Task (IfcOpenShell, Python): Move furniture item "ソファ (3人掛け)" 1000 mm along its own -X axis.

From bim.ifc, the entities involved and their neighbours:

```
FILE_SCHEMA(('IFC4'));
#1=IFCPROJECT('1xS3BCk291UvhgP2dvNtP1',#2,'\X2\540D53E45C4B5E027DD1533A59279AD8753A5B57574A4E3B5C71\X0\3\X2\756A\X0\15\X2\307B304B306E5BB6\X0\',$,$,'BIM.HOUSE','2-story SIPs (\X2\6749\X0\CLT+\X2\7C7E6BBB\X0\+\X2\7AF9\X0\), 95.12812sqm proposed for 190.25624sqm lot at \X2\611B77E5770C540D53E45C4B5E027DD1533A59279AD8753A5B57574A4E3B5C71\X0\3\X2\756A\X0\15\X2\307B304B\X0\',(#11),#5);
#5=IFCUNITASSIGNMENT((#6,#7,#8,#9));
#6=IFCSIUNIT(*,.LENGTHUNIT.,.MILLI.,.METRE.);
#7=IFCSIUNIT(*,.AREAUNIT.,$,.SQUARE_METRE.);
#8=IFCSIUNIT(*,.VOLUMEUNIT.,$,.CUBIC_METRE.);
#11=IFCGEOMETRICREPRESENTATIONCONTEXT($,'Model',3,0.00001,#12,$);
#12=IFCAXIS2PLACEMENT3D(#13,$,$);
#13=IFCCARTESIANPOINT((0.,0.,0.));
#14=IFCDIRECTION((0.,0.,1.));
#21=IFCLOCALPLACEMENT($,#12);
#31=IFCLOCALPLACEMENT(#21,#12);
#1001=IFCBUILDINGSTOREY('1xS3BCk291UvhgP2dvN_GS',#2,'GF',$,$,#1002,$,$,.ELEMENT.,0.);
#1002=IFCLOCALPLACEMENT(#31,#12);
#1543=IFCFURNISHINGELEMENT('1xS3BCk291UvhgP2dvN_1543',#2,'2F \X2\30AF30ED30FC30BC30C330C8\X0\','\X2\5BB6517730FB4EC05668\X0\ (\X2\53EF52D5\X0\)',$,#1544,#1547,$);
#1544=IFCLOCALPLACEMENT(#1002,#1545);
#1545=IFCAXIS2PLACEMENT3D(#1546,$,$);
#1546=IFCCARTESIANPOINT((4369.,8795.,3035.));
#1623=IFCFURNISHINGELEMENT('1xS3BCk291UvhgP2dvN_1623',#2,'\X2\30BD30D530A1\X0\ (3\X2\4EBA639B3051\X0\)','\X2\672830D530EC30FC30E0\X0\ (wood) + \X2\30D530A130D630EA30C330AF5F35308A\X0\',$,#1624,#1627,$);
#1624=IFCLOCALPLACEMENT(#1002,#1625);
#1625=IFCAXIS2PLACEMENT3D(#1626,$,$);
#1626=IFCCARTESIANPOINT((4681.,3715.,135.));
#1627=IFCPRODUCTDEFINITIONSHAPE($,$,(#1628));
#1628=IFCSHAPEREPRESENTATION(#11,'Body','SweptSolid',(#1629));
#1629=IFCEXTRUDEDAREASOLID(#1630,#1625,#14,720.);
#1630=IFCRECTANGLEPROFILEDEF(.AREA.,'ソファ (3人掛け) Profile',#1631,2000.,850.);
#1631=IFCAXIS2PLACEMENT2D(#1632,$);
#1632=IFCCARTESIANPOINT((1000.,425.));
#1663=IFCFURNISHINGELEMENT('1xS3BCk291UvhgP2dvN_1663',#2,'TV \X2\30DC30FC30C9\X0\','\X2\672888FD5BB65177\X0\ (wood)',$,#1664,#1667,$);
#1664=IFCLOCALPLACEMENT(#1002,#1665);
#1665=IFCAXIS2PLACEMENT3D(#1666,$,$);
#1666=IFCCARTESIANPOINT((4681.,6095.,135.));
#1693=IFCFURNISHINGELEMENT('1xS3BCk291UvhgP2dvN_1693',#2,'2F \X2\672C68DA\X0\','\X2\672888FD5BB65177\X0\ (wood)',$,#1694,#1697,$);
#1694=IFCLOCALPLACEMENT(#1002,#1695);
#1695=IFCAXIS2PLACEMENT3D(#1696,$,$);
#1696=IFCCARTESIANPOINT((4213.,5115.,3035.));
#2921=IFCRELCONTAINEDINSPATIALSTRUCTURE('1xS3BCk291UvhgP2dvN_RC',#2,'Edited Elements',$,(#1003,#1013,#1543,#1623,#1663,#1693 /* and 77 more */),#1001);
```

```python
import ifcopenshell
import ifcopenshell.api.geometry
import ifcopenshell.util.placement

model = ifcopenshell.open("bim.ifc")

item = model.by_id(1623)
matrix = ifcopenshell.util.placement.get_local_placement(item.ObjectPlacement)
matrix[:3, 3] -= matrix[:3, 0] * 1000.0
ifcopenshell.api.geometry.edit_object_placement(model, product=item, matrix=matrix, is_si=False)

print(ifcopenshell.util.placement.get_local_placement(item.ObjectPlacement).round(3) + 0.0)

model.write("bim-out.ifc")
```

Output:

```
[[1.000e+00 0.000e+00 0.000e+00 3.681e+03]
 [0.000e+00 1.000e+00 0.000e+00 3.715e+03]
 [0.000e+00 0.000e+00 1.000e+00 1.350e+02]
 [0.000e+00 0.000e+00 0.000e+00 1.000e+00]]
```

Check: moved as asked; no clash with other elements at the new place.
